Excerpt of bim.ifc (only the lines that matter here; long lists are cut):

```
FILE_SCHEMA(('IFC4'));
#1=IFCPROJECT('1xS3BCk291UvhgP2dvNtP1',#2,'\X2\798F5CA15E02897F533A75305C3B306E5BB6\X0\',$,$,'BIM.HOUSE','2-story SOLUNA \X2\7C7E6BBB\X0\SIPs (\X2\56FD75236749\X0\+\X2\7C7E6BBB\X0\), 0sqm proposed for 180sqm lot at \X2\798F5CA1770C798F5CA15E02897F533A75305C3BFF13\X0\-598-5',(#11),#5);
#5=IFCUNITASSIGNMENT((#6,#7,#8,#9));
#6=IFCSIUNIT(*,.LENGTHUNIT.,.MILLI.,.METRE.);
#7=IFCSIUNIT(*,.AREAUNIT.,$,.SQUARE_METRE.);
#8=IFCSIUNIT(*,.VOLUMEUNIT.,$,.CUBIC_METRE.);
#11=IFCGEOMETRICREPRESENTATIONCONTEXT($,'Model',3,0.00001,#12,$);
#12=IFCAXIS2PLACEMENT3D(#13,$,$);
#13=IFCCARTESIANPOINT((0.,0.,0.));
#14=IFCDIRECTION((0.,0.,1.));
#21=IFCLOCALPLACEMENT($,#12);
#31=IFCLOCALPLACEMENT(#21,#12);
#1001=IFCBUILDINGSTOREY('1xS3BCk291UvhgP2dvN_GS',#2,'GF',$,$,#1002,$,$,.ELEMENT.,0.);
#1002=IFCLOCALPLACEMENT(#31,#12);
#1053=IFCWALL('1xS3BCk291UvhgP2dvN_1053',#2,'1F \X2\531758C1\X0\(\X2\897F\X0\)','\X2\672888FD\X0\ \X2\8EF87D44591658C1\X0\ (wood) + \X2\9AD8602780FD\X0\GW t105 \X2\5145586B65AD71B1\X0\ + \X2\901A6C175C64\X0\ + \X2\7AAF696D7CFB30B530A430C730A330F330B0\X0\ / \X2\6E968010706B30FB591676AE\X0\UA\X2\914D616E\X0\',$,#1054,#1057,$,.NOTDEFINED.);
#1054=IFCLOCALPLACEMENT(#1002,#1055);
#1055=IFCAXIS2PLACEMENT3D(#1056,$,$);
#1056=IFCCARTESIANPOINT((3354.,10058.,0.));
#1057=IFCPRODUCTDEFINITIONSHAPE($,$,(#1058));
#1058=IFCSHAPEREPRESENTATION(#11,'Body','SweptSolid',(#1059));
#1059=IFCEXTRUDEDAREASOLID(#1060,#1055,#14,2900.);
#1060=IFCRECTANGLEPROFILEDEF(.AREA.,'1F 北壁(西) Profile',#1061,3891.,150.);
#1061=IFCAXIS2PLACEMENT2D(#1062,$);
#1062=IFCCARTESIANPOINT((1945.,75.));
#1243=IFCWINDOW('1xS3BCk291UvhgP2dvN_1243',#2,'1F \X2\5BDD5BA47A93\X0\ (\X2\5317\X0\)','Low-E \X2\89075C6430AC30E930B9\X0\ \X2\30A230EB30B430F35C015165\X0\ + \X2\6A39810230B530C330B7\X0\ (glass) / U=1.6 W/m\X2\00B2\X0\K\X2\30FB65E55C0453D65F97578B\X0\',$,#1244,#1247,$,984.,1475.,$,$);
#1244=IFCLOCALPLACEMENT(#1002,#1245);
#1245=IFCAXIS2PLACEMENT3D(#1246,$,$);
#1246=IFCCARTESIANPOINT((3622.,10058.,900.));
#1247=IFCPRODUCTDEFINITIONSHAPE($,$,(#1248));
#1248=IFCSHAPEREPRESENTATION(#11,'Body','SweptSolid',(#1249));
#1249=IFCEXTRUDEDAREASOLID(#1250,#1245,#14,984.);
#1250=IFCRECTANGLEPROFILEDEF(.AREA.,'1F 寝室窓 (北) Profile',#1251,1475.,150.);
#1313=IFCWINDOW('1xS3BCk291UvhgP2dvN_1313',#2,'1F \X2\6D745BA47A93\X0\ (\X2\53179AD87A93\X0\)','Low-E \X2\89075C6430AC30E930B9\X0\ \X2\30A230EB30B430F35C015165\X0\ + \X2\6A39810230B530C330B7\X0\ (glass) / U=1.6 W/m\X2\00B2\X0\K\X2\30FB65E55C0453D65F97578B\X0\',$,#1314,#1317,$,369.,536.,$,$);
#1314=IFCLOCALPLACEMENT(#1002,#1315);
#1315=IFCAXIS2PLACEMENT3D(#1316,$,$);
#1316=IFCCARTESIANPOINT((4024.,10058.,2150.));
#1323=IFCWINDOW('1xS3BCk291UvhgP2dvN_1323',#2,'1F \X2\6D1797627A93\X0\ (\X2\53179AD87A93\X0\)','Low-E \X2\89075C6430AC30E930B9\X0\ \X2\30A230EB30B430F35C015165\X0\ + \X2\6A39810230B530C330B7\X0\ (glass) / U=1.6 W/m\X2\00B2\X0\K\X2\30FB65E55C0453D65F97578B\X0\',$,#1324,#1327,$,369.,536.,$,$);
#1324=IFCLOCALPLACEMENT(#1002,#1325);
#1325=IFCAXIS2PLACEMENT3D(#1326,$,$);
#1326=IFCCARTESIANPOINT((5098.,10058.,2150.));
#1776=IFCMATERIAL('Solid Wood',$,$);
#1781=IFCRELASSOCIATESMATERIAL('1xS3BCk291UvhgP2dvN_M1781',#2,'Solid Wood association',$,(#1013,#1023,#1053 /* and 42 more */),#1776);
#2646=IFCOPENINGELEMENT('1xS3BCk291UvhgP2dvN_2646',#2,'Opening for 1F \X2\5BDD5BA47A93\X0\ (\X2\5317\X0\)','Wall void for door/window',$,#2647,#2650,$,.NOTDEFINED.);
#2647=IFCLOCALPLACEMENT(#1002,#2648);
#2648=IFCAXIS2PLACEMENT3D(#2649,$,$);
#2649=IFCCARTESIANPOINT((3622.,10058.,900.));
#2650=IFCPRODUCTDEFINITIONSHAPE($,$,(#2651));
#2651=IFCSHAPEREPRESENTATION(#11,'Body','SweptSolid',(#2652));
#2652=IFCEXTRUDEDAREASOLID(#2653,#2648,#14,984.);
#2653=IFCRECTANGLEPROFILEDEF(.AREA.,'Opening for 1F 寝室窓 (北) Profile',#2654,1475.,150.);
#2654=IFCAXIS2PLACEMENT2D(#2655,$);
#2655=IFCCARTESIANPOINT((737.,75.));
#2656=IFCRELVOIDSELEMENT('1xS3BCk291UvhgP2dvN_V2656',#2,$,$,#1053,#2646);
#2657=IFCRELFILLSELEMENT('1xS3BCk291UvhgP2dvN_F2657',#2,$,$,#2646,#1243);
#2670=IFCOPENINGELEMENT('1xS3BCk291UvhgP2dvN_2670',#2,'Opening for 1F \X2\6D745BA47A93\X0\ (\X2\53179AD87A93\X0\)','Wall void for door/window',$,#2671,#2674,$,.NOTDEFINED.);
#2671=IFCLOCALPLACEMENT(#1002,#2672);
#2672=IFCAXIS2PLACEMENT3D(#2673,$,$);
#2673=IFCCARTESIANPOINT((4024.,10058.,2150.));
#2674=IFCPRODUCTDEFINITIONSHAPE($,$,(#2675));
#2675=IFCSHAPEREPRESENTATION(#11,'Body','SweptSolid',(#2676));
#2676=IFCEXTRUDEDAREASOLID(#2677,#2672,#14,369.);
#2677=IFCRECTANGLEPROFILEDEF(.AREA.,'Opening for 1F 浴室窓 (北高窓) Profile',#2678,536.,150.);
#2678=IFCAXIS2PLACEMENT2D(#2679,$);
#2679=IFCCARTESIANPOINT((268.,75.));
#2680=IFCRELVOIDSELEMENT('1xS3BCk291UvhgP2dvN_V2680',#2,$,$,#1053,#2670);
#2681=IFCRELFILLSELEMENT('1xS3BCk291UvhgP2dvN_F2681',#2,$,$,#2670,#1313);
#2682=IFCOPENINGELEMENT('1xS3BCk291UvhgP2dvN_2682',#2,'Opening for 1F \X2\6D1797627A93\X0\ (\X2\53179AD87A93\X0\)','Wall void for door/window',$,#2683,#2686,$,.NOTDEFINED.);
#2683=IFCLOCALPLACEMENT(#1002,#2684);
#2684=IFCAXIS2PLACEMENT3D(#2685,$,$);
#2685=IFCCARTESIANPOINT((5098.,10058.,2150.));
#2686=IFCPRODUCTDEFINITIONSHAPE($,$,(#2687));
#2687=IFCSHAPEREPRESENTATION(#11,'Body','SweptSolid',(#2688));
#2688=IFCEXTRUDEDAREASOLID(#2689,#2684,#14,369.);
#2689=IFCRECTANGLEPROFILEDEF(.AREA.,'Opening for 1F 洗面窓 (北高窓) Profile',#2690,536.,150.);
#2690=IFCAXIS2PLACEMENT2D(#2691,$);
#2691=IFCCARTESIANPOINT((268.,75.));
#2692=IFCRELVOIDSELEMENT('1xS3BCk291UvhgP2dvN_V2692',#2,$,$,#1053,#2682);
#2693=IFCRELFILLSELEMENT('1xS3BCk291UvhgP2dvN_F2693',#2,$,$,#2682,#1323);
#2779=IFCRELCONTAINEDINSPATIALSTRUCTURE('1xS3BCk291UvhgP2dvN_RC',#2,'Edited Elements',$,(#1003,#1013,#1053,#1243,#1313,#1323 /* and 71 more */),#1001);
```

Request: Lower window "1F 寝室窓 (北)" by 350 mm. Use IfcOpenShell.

```python
import numpy as np
import ifcopenshell
import ifcopenshell.api.geometry
import ifcopenshell.util.placement
import ifcopenshell.util.unit

model = ifcopenshell.open("bim.ifc")
unit_scale = ifcopenshell.util.unit.calculate_unit_scale(model)

window = model.by_id(1243)
opening = window.FillsVoids[0].RelatingOpeningElement
dz = -350.0

shift = np.array([0.0, 0.0, dz])
# The window is not placed relative to its opening, so move both.
for product in (opening, window):
    matrix = ifcopenshell.util.placement.get_local_placement(product.ObjectPlacement)
    matrix[:3, 3] += shift
    ifcopenshell.api.geometry.edit_object_placement(model, product=product, matrix=matrix, is_si=False)

print(f"moved by {dz * unit_scale:+.3f} m")

model.write("bim_v2.ifc")
```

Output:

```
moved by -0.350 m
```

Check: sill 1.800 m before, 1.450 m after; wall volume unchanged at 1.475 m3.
